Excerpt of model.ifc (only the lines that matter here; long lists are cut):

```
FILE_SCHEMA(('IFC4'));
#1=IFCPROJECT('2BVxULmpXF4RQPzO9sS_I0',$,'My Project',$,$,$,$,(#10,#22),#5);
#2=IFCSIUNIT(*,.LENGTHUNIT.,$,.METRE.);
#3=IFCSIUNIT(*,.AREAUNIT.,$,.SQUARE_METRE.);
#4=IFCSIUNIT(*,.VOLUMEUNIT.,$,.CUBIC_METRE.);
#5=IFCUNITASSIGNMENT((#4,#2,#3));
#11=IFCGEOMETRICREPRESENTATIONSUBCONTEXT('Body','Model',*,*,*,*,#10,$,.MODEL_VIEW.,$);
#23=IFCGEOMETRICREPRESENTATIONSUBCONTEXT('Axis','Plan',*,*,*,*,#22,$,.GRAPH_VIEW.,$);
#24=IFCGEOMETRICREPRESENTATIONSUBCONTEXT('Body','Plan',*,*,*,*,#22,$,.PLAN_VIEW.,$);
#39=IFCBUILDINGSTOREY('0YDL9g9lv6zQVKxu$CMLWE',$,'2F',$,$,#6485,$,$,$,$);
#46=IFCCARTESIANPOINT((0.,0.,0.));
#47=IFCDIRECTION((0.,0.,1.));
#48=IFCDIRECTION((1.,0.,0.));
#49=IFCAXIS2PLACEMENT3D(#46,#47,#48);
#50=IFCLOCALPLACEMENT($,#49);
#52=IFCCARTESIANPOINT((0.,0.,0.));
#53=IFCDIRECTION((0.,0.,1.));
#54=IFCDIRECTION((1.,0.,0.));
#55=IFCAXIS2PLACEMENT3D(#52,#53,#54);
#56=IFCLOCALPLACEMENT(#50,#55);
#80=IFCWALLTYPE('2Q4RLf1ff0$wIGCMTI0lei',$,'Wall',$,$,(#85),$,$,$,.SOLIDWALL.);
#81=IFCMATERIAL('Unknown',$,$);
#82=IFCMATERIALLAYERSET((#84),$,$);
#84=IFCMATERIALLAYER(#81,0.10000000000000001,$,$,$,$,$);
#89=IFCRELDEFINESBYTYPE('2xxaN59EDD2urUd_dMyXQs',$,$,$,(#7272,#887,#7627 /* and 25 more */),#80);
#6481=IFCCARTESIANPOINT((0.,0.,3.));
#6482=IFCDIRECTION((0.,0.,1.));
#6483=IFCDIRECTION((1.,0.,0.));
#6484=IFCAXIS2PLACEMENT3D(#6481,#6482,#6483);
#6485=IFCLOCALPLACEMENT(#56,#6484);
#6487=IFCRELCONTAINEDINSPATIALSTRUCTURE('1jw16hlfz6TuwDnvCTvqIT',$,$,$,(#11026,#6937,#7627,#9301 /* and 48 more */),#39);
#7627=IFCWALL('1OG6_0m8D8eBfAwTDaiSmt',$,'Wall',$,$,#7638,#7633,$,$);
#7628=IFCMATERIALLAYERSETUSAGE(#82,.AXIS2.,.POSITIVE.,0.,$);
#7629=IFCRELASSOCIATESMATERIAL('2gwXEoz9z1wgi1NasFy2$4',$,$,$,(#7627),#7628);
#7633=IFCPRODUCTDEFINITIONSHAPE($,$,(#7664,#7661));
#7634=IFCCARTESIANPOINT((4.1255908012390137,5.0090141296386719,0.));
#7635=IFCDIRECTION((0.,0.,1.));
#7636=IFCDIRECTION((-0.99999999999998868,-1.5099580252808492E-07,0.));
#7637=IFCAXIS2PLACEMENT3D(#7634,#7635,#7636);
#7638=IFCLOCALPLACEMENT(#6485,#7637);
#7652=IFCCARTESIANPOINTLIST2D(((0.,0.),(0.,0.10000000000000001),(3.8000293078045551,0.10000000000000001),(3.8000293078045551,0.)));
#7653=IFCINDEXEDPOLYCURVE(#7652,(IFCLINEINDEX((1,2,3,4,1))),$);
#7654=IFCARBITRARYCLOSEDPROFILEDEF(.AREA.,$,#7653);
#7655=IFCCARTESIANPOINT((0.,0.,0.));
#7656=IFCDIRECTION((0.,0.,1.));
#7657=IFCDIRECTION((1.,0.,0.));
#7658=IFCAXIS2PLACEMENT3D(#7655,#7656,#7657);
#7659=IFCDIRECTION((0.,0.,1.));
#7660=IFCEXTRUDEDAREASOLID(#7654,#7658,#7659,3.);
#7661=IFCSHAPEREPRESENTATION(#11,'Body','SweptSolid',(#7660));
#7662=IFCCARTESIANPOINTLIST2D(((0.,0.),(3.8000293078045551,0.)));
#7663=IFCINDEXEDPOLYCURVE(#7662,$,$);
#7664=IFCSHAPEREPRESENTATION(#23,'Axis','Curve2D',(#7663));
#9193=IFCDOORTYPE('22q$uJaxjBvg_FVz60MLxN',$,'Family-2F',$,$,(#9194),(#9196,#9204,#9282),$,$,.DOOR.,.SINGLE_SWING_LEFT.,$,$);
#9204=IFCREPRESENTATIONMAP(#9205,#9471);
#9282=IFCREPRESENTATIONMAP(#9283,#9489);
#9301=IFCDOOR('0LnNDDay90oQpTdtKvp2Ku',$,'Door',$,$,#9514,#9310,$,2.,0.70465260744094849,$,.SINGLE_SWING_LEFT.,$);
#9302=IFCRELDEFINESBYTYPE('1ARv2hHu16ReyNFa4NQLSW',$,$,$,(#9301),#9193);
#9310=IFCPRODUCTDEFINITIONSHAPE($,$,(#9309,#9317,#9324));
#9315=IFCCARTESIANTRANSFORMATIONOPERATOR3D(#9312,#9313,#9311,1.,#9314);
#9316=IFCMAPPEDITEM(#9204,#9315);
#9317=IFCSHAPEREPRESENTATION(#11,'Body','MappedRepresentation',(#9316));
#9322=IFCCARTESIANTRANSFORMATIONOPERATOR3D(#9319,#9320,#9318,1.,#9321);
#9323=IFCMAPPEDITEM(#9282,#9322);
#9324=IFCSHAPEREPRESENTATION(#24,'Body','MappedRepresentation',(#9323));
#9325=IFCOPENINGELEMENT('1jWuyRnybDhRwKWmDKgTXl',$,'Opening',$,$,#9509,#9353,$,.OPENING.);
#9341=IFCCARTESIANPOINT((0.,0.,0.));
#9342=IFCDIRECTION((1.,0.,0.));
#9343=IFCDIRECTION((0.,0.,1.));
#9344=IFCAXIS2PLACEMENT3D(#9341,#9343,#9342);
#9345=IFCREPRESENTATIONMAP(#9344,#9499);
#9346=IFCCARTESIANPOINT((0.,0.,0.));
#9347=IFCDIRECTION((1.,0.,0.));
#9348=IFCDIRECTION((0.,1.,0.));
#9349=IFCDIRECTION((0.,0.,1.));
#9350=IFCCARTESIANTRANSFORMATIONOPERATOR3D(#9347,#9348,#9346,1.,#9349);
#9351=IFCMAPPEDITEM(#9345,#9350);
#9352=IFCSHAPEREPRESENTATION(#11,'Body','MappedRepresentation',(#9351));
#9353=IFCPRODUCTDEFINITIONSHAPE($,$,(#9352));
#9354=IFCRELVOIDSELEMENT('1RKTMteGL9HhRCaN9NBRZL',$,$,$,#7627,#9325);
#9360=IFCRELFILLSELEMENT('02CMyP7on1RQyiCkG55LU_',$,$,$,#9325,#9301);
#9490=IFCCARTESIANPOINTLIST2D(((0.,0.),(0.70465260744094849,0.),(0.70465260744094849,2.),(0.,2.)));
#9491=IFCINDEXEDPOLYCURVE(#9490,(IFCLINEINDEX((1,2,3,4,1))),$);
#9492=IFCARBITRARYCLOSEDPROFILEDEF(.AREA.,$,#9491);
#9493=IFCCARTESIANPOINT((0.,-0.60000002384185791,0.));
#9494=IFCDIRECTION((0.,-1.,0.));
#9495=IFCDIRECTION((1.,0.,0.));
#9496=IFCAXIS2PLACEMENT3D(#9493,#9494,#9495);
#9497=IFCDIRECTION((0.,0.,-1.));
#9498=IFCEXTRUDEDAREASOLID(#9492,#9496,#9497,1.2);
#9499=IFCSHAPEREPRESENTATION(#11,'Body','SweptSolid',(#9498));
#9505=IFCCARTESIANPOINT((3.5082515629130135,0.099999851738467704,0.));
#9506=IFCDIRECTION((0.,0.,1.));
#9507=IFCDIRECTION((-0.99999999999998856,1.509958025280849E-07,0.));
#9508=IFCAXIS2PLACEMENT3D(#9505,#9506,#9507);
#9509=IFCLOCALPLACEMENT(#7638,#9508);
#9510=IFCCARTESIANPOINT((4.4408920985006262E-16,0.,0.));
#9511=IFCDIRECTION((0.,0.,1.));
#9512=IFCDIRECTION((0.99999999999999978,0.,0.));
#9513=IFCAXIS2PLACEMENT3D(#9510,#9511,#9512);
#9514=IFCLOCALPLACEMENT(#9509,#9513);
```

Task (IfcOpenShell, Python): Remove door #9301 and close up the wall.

```python
import ifcopenshell
import ifcopenshell.api.feature
import ifcopenshell.api.root
import ifcopenshell.geom
import ifcopenshell.util.shape

model = ifcopenshell.open("model.ifc")
settings = ifcopenshell.geom.settings()


def volume(element):
    """Net volume in cubic metres, openings subtracted."""
    shape = ifcopenshell.geom.create_shape(settings, element)
    return ifcopenshell.util.shape.get_volume(shape.geometry)


door = model.by_guid("0LnNDDay90oQpTdtKvp2Ku")
opening = door.FillsVoids[0].RelatingOpeningElement
wall = opening.VoidsElements[0].RelatingBuildingElement
before = volume(wall)

ifcopenshell.api.root.remove_product(model, product=door)
ifcopenshell.api.feature.remove_feature(model, feature=opening)

after = volume(wall)

print(f"wall volume {before:.3f} -> {after:.3f} m3")

model.write("model_rev.ifc")
```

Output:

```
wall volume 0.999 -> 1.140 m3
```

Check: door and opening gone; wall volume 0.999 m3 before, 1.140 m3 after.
